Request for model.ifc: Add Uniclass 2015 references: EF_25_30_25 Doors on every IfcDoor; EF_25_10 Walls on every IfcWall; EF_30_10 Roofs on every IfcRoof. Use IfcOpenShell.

First a look at what the model holds.

```python
import ifcopenshell

model = ifcopenshell.open("model.ifc")
print(model.schema)
print("classifications:", [c.Name for c in model.by_type("IfcClassification")])
for ifc_class in ("IfcDoor", "IfcRoof", "IfcStair", "IfcWall", "IfcWindow"):
    print(ifc_class, len(model.by_type(ifc_class)))
```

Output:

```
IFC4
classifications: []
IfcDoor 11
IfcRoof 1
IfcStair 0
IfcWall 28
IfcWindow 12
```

```python
import ifcopenshell
import ifcopenshell.api.classification

model = ifcopenshell.open("model.ifc")

system = ifcopenshell.api.classification.add_classification(model, classification="Uniclass 2015")

codes = {
    "IfcDoor": ("EF_25_30_25", "Doors"),
    "IfcWall": ("EF_25_10", "Walls"),
    "IfcRoof": ("EF_30_10", "Roofs"),
}
for ifc_class, (code, name) in codes.items():
    products = model.by_type(ifc_class)
    ifcopenshell.api.classification.add_reference(
        model, products=products, classification=system, identification=code, name=name
    )
    print(code, len(products))

model.write("model_rev.ifc")
```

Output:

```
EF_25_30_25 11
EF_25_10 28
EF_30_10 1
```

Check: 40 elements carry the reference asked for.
